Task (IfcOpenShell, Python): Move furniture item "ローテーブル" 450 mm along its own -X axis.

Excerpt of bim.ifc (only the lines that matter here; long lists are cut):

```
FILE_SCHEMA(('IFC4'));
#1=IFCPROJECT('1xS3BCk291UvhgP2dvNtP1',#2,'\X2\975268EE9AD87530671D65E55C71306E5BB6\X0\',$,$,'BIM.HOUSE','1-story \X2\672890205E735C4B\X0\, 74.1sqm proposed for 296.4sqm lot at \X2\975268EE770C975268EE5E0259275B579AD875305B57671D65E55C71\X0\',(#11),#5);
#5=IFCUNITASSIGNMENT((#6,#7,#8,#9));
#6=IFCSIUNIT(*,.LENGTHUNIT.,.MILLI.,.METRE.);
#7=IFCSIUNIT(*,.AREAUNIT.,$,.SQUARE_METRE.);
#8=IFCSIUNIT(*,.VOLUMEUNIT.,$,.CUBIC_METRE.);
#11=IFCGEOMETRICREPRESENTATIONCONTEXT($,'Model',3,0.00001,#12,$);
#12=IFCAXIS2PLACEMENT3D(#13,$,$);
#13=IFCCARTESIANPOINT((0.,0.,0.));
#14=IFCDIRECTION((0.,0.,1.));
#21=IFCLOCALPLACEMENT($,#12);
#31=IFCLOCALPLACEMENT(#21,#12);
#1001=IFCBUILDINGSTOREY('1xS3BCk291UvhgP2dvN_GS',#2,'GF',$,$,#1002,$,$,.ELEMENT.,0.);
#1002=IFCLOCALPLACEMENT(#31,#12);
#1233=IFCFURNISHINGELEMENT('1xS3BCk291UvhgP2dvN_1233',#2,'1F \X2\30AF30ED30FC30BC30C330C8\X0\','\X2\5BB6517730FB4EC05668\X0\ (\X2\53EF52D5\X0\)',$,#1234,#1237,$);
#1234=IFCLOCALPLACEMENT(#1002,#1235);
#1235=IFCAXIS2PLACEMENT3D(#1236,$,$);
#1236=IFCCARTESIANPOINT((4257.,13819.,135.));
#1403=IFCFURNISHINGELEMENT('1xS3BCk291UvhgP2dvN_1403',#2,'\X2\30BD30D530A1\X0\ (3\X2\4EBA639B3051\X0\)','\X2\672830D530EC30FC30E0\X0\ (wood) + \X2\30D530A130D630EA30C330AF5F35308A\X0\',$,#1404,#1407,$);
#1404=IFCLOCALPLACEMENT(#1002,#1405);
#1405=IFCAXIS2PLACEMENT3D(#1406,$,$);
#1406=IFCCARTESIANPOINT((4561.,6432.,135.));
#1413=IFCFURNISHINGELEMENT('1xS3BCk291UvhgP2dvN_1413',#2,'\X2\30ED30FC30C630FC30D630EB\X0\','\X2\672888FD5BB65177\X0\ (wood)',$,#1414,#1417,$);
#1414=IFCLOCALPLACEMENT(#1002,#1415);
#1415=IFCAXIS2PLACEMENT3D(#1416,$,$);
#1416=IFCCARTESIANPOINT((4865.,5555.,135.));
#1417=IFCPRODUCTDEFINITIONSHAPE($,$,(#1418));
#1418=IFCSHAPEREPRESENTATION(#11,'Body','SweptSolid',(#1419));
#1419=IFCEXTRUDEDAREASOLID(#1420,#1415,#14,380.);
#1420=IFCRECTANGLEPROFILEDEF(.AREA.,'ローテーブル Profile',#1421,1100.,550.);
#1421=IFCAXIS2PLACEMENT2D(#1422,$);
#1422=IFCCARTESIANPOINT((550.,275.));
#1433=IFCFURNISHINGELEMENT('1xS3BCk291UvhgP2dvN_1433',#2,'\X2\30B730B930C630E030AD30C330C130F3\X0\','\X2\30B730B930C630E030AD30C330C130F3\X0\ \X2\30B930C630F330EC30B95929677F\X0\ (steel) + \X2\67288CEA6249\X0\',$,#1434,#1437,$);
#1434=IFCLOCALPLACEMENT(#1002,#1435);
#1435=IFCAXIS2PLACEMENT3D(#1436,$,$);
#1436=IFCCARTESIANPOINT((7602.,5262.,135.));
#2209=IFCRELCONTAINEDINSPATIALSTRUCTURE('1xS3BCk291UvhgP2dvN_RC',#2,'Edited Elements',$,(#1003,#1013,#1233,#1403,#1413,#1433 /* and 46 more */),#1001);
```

```python
import ifcopenshell
import ifcopenshell.api.geometry
import ifcopenshell.util.placement
import ifcopenshell.util.unit

model = ifcopenshell.open("bim.ifc")
unit_scale = ifcopenshell.util.unit.calculate_unit_scale(model)

item = model.by_id(1413)
matrix = ifcopenshell.util.placement.get_local_placement(item.ObjectPlacement)
matrix[:3, 3] -= matrix[:3, 0] * 0.45 / unit_scale
ifcopenshell.api.geometry.edit_object_placement(model, product=item, matrix=matrix, is_si=False)

print(ifcopenshell.util.placement.get_local_placement(item.ObjectPlacement).round(3) + 0.0)

model.write("bim_v2.ifc")
```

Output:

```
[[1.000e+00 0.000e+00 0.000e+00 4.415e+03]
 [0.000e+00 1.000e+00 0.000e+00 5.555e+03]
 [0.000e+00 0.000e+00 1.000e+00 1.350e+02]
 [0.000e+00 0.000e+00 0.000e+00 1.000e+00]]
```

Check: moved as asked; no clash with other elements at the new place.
